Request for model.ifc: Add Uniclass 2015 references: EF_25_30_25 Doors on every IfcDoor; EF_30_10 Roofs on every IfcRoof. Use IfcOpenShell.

First a look at what the model holds.

```python
import ifcopenshell

model = ifcopenshell.open("model.ifc")
print(model.schema)
print("classifications:", [c.Name for c in model.by_type("IfcClassification")])
for ifc_class in ("IfcDoor", "IfcRoof", "IfcStair", "IfcWall", "IfcWindow"):
    print(ifc_class, len(model.by_type(ifc_class)))
```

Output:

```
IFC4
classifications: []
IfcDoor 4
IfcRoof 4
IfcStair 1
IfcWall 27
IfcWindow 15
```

```python
import ifcopenshell
import ifcopenshell.api.classification

model = ifcopenshell.open("model.ifc")

system = ifcopenshell.api.classification.add_classification(model, classification="Uniclass 2015")

codes = {
    "IfcDoor": ("EF_25_30_25", "Doors"),
    "IfcRoof": ("EF_30_10", "Roofs"),
}
for ifc_class, (code, name) in codes.items():
    products = model.by_type(ifc_class)
    ifcopenshell.api.classification.add_reference(
        model, products=products, classification=system, identification=code, name=name
    )
    print(code, len(products))

model.write("model_updated.ifc")
```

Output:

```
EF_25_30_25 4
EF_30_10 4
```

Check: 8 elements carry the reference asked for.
